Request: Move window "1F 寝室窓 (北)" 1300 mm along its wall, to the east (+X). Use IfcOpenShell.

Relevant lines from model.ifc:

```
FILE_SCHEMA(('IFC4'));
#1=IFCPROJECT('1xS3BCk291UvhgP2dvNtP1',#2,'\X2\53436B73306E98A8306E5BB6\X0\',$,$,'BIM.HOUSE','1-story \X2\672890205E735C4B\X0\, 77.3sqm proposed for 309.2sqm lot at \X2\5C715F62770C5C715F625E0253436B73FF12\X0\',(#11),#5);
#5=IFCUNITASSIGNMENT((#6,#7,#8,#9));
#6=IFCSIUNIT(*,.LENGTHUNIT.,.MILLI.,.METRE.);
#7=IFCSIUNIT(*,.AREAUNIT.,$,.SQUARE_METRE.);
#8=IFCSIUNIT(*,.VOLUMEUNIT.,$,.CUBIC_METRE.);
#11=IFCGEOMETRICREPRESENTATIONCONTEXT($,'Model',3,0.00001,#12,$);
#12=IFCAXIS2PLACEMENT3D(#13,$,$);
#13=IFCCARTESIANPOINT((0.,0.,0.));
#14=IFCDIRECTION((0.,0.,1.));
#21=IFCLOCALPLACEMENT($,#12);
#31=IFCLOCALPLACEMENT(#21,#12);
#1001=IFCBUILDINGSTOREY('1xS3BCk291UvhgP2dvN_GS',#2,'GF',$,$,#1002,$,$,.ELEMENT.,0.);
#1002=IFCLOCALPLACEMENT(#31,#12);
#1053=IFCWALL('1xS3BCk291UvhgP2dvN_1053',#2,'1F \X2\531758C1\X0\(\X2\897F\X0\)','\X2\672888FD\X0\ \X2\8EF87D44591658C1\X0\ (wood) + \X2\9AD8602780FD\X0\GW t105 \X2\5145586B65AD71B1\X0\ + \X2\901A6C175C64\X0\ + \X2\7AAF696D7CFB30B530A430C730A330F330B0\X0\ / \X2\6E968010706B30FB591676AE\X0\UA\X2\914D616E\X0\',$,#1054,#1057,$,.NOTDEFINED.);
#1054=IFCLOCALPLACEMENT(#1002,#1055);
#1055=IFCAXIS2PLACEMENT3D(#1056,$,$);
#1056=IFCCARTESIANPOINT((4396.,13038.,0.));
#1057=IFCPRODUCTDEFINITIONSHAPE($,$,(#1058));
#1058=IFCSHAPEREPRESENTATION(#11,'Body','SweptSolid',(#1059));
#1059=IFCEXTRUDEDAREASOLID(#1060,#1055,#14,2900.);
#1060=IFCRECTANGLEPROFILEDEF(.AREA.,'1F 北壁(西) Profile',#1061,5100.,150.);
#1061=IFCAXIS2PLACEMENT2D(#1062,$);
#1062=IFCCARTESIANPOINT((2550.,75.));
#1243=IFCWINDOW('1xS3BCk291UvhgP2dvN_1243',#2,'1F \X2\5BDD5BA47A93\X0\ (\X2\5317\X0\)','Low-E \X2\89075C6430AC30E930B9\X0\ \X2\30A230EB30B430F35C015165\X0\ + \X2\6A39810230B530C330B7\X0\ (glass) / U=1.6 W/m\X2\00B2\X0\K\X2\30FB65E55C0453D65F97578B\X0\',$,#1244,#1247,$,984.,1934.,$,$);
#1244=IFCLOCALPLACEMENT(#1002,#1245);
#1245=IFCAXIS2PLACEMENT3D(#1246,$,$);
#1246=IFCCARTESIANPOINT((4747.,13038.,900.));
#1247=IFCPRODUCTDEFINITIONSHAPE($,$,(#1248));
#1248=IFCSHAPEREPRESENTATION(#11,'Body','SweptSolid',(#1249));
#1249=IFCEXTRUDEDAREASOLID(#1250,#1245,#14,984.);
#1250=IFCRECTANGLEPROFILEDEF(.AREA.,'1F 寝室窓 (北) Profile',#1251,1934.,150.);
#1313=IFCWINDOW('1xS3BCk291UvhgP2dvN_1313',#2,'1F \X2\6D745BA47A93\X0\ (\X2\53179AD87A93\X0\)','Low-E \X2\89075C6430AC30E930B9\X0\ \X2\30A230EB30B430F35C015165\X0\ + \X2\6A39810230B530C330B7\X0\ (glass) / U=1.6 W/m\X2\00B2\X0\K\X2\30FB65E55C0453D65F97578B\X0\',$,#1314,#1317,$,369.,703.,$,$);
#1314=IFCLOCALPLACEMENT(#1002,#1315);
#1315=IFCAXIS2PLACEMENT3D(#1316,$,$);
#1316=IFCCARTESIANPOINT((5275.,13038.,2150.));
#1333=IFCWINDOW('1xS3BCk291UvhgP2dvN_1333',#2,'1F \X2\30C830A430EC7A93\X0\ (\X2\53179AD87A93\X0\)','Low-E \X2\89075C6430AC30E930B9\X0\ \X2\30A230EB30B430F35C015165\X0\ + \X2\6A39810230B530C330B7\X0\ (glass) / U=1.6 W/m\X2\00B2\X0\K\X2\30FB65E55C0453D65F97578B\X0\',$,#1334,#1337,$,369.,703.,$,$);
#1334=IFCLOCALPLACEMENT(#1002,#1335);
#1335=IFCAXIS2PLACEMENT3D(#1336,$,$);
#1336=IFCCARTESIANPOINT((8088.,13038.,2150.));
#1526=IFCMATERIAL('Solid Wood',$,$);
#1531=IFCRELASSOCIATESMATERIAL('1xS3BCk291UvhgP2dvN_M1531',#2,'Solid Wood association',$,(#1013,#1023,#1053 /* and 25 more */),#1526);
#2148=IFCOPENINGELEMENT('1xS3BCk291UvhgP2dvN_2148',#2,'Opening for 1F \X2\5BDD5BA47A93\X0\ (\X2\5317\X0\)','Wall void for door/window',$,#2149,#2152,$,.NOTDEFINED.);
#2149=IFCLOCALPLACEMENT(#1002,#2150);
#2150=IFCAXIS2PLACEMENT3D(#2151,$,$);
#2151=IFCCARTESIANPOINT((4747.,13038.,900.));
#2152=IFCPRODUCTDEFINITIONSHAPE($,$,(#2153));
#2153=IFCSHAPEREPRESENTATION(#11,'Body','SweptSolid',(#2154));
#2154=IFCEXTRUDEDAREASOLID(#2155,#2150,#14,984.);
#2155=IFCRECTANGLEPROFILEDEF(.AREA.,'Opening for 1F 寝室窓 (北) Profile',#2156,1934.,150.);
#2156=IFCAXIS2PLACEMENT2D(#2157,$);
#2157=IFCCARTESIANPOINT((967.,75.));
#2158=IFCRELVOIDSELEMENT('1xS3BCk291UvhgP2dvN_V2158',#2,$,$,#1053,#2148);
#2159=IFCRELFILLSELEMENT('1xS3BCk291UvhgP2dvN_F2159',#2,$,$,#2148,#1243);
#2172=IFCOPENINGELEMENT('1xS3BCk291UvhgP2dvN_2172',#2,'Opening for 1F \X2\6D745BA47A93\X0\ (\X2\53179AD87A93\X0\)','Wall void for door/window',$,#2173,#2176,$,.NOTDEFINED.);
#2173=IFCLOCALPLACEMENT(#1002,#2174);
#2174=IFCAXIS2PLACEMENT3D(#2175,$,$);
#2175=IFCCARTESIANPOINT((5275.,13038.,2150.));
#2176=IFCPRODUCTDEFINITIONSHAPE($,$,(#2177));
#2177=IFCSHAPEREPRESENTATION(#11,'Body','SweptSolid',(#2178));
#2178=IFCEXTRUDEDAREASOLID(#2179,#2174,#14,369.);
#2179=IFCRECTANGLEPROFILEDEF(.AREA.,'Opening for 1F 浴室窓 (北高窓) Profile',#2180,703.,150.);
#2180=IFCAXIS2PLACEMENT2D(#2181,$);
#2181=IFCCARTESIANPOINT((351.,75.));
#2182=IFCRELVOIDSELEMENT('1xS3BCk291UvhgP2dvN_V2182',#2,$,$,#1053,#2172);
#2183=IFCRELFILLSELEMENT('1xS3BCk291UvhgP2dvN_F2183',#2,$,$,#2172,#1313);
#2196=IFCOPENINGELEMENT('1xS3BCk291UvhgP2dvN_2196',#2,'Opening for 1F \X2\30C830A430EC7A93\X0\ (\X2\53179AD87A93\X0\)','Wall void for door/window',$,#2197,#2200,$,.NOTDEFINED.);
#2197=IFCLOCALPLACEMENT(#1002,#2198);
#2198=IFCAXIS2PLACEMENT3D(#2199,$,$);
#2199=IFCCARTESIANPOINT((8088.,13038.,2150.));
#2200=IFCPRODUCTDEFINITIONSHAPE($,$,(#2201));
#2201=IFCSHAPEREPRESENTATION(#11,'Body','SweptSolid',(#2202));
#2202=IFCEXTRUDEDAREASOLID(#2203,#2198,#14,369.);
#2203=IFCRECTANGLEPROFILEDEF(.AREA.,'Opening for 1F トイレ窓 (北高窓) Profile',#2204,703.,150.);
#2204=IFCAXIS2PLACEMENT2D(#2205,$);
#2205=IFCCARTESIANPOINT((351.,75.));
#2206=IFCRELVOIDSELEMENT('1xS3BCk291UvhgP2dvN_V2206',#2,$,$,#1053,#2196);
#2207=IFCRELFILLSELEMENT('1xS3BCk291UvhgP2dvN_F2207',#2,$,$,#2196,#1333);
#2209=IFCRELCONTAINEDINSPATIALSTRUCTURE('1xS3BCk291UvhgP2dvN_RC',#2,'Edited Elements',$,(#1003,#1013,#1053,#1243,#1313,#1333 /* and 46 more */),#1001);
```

```python
import ifcopenshell
import ifcopenshell.api.geometry
import ifcopenshell.util.placement
import ifcopenshell.util.unit

model = ifcopenshell.open("model.ifc")
unit_scale = ifcopenshell.util.unit.calculate_unit_scale(model)

window = model.by_guid("1xS3BCk291UvhgP2dvN_1243")
opening = window.FillsVoids[0].RelatingOpeningElement
wall = opening.VoidsElements[0].RelatingBuildingElement

wall_matrix = ifcopenshell.util.placement.get_local_placement(wall.ObjectPlacement)
shift = wall_matrix[:3, 0] * 1.3 / unit_scale
before = ifcopenshell.util.placement.get_local_placement(window.ObjectPlacement)[:3, 3].copy()

# The window is not placed relative to its opening, so move both.
for product in (opening, window):
    matrix = ifcopenshell.util.placement.get_local_placement(product.ObjectPlacement)
    matrix[:3, 3] += shift
    ifcopenshell.api.geometry.edit_object_placement(model, product=product, matrix=matrix, is_si=False)

after = ifcopenshell.util.placement.get_local_placement(window.ObjectPlacement)[:3, 3]
print("window moved by", (after - before).round(3) + 0.0)

model.write("model-out.ifc")
```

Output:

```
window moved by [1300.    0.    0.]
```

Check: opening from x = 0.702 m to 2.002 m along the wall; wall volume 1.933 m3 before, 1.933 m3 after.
